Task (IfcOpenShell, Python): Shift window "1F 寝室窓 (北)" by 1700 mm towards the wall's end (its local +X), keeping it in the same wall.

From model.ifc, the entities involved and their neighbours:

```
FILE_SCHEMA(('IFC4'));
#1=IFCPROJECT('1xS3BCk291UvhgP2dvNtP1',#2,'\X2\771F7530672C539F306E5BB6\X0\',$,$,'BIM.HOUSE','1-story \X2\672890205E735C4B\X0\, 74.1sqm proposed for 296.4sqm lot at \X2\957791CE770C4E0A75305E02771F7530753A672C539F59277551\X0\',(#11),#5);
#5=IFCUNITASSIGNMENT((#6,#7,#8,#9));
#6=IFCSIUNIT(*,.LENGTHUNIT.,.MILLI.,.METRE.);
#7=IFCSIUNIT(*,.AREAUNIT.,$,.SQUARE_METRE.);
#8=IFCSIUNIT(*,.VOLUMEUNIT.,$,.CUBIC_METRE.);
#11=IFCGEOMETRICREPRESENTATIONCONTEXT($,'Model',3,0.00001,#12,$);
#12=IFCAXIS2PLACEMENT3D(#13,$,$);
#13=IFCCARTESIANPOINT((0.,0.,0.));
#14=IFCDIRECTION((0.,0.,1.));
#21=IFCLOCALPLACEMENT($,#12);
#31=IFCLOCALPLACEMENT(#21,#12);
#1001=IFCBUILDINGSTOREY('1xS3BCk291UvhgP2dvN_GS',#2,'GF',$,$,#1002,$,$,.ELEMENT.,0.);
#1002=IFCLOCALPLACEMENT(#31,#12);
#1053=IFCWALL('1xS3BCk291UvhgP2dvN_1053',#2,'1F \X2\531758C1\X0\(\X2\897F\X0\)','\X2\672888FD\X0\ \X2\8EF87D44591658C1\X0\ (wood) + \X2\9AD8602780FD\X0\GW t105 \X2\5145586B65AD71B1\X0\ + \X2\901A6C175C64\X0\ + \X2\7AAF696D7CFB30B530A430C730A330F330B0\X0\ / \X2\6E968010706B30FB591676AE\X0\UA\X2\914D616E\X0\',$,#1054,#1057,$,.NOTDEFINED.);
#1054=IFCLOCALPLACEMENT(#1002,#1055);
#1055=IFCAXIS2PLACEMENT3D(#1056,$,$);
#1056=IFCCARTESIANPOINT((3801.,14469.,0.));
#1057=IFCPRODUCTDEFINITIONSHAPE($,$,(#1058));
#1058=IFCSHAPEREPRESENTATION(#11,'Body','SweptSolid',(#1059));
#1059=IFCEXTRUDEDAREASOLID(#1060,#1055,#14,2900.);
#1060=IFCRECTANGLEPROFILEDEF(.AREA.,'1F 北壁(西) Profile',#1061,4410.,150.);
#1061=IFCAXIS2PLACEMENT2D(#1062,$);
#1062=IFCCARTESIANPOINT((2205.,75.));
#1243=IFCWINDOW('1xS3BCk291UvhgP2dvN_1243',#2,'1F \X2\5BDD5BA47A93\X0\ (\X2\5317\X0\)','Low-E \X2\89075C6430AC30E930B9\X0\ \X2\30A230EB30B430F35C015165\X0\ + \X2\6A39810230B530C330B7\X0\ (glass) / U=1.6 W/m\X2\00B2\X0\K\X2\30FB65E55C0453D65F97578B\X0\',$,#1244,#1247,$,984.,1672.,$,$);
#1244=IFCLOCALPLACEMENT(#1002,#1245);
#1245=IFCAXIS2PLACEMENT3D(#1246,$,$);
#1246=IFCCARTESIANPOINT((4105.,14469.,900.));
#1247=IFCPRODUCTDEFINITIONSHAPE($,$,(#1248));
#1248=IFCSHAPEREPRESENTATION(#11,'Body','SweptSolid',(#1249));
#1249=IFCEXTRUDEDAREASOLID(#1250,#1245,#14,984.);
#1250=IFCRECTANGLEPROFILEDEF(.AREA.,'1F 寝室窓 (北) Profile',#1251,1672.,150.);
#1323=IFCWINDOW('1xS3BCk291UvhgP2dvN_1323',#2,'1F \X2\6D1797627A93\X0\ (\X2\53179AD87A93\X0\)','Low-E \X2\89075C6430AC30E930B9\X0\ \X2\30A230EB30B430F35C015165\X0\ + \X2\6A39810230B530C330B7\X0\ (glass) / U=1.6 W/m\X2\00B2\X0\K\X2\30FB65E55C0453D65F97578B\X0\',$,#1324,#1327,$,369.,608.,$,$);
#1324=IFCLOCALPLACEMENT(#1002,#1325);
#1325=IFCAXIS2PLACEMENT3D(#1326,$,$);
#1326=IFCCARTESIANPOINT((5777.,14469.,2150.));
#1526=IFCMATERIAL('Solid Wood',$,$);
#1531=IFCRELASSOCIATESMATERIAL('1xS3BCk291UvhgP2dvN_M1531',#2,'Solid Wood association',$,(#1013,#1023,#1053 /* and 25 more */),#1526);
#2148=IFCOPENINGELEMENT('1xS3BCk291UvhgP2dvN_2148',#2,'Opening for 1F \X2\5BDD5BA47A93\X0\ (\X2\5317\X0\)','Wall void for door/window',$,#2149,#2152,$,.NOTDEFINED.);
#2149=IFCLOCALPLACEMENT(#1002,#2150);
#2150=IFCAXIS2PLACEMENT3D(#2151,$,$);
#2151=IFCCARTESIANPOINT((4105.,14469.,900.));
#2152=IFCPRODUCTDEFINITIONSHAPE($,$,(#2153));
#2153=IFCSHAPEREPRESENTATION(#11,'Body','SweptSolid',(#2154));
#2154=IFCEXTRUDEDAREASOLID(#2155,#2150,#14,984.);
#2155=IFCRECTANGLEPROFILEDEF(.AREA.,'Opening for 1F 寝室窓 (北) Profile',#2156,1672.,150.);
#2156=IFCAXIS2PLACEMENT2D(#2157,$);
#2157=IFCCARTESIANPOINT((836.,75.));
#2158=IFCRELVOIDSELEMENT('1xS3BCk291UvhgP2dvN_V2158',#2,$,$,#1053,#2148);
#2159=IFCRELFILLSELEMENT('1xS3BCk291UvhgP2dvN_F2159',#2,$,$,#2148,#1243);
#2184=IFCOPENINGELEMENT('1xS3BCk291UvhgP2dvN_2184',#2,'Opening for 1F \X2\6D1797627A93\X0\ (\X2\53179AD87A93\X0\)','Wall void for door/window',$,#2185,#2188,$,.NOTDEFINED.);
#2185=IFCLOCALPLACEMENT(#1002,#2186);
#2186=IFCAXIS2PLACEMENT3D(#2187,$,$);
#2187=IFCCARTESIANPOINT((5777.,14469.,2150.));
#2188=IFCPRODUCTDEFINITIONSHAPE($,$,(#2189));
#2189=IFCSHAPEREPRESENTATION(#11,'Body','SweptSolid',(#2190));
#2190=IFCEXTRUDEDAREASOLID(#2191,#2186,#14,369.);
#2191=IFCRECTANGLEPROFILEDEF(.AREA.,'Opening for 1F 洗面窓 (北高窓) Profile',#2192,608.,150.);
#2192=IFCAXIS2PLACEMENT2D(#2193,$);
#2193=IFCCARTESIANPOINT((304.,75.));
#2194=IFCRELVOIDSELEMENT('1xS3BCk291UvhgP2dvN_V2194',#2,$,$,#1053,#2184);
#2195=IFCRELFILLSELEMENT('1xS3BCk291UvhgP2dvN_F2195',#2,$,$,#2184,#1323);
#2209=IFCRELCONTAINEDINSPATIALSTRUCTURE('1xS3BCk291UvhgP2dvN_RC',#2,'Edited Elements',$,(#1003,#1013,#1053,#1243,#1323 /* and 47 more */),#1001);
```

```python
import ifcopenshell
import ifcopenshell.api.geometry
import ifcopenshell.util.placement
import ifcopenshell.util.unit

model = ifcopenshell.open("model.ifc")
unit_scale = ifcopenshell.util.unit.calculate_unit_scale(model)

window = model.by_guid("1xS3BCk291UvhgP2dvN_1243")
opening = window.FillsVoids[0].RelatingOpeningElement
wall = opening.VoidsElements[0].RelatingBuildingElement

wall_matrix = ifcopenshell.util.placement.get_local_placement(wall.ObjectPlacement)
shift = wall_matrix[:3, 0] * 1.7 / unit_scale
before = ifcopenshell.util.placement.get_local_placement(window.ObjectPlacement)[:3, 3].copy()

# The window is not placed relative to its opening, so move both.
for product in (opening, window):
    matrix = ifcopenshell.util.placement.get_local_placement(product.ObjectPlacement)
    matrix[:3, 3] += shift
    ifcopenshell.api.geometry.edit_object_placement(model, product=product, matrix=matrix, is_si=False)

after = ifcopenshell.util.placement.get_local_placement(window.ObjectPlacement)[:3, 3]
print("window moved by", (after - before).round(3) + 0.0)

model.write("model_v2.ifc")
```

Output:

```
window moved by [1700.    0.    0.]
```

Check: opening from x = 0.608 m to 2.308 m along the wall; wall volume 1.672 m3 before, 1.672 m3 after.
